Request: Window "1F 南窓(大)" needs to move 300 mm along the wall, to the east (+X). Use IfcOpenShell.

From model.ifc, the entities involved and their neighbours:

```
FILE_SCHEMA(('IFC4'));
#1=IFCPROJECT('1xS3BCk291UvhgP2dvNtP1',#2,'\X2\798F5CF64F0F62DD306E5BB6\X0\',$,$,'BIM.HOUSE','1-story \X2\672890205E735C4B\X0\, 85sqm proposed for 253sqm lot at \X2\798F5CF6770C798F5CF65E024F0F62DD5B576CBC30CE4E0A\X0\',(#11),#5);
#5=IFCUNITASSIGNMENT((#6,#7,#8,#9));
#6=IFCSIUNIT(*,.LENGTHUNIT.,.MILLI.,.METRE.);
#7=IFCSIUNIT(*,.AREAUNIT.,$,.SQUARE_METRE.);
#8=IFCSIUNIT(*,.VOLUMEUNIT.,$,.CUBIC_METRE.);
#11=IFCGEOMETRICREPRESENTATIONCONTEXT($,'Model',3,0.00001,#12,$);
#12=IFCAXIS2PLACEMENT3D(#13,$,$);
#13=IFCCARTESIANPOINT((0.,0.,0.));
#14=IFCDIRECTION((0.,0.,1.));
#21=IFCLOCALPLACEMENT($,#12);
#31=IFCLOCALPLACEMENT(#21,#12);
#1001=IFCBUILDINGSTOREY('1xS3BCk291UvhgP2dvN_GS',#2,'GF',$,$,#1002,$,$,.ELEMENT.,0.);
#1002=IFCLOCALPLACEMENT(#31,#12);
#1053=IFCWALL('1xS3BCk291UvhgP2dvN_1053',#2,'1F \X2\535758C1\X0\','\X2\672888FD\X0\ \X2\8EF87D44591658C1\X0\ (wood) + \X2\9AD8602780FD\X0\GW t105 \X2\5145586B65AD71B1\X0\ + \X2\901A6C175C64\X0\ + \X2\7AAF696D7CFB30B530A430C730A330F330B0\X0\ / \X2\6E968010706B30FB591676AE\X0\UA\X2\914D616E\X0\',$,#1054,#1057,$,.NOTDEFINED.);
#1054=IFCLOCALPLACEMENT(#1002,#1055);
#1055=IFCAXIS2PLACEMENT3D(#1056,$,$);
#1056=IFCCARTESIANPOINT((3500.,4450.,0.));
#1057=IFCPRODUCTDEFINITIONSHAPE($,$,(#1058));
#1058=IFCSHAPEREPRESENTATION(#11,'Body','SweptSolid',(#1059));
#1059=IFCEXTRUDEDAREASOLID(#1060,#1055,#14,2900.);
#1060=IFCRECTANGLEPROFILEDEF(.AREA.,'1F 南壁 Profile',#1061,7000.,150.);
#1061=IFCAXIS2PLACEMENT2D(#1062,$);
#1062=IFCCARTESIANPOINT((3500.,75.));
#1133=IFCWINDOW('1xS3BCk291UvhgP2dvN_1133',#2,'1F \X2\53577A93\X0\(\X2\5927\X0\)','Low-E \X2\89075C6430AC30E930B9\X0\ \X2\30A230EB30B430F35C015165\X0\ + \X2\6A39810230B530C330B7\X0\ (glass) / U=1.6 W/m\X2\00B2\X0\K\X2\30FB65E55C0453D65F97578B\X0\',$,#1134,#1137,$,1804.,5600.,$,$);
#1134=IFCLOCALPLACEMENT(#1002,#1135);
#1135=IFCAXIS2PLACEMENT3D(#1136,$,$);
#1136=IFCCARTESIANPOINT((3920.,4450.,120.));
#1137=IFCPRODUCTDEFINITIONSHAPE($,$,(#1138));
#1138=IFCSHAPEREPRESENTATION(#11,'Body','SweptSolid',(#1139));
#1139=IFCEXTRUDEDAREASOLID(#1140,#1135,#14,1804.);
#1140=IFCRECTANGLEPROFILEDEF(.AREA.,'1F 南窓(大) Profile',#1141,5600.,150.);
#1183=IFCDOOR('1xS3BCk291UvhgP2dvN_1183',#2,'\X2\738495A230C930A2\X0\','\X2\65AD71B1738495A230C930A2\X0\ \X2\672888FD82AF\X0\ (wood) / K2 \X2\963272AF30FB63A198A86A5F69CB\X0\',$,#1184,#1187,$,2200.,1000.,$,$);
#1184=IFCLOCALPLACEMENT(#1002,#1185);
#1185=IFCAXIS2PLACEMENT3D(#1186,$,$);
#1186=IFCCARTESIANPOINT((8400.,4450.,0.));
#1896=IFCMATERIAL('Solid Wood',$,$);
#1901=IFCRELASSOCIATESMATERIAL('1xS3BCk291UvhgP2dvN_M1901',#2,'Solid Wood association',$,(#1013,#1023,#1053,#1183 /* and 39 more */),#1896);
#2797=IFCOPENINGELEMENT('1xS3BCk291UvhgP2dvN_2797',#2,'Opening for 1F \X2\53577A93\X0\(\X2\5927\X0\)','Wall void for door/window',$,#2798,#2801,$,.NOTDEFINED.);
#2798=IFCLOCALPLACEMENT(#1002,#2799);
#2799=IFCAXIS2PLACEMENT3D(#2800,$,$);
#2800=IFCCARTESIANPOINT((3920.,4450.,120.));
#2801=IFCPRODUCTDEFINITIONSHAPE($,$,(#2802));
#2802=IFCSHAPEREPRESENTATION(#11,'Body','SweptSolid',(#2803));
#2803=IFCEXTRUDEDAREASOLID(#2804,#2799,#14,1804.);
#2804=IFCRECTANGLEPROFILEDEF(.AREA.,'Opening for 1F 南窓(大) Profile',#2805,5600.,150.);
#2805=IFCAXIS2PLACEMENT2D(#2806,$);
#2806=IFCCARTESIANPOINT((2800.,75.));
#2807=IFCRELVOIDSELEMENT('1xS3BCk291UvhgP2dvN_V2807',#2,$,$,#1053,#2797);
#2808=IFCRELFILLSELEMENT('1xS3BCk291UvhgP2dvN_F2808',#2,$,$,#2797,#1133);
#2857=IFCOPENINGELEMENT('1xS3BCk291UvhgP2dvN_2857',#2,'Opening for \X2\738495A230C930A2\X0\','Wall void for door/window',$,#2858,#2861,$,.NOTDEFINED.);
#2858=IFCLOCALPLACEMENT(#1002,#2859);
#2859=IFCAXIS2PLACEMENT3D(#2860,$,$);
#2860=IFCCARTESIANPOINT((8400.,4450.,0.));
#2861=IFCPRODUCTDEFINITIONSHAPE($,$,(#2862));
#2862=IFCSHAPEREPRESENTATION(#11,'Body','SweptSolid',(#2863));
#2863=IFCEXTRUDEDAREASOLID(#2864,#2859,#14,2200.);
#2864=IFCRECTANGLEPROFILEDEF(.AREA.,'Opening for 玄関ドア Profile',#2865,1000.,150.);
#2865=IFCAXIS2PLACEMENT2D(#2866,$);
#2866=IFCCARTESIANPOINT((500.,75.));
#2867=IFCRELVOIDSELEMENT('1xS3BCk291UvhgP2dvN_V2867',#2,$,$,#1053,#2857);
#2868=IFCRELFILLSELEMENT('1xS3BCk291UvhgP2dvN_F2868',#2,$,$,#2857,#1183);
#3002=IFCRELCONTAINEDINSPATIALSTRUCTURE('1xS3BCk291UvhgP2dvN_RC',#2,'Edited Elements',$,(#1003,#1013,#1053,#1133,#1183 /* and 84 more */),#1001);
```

```python
import ifcopenshell
import ifcopenshell.api.geometry
import ifcopenshell.util.placement
import ifcopenshell.util.unit

model = ifcopenshell.open("model.ifc")
unit_scale = ifcopenshell.util.unit.calculate_unit_scale(model)

window = model.by_id(1133)
opening = window.FillsVoids[0].RelatingOpeningElement
wall = opening.VoidsElements[0].RelatingBuildingElement

wall_matrix = ifcopenshell.util.placement.get_local_placement(wall.ObjectPlacement)
shift = wall_matrix[:3, 0] * 0.3 / unit_scale
before = ifcopenshell.util.placement.get_local_placement(window.ObjectPlacement)[:3, 3].copy()

# The window is not placed relative to its opening, so move both.
for product in (opening, window):
    matrix = ifcopenshell.util.placement.get_local_placement(product.ObjectPlacement)
    matrix[:3, 3] += shift
    ifcopenshell.api.geometry.edit_object_placement(model, product=product, matrix=matrix, is_si=False)

after = ifcopenshell.util.placement.get_local_placement(window.ObjectPlacement)[:3, 3]
print("window moved by", (after - before).round(3) + 0.0)

model.write("model_edited.ifc")
```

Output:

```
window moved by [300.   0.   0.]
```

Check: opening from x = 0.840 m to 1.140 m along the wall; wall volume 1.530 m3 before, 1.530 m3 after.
